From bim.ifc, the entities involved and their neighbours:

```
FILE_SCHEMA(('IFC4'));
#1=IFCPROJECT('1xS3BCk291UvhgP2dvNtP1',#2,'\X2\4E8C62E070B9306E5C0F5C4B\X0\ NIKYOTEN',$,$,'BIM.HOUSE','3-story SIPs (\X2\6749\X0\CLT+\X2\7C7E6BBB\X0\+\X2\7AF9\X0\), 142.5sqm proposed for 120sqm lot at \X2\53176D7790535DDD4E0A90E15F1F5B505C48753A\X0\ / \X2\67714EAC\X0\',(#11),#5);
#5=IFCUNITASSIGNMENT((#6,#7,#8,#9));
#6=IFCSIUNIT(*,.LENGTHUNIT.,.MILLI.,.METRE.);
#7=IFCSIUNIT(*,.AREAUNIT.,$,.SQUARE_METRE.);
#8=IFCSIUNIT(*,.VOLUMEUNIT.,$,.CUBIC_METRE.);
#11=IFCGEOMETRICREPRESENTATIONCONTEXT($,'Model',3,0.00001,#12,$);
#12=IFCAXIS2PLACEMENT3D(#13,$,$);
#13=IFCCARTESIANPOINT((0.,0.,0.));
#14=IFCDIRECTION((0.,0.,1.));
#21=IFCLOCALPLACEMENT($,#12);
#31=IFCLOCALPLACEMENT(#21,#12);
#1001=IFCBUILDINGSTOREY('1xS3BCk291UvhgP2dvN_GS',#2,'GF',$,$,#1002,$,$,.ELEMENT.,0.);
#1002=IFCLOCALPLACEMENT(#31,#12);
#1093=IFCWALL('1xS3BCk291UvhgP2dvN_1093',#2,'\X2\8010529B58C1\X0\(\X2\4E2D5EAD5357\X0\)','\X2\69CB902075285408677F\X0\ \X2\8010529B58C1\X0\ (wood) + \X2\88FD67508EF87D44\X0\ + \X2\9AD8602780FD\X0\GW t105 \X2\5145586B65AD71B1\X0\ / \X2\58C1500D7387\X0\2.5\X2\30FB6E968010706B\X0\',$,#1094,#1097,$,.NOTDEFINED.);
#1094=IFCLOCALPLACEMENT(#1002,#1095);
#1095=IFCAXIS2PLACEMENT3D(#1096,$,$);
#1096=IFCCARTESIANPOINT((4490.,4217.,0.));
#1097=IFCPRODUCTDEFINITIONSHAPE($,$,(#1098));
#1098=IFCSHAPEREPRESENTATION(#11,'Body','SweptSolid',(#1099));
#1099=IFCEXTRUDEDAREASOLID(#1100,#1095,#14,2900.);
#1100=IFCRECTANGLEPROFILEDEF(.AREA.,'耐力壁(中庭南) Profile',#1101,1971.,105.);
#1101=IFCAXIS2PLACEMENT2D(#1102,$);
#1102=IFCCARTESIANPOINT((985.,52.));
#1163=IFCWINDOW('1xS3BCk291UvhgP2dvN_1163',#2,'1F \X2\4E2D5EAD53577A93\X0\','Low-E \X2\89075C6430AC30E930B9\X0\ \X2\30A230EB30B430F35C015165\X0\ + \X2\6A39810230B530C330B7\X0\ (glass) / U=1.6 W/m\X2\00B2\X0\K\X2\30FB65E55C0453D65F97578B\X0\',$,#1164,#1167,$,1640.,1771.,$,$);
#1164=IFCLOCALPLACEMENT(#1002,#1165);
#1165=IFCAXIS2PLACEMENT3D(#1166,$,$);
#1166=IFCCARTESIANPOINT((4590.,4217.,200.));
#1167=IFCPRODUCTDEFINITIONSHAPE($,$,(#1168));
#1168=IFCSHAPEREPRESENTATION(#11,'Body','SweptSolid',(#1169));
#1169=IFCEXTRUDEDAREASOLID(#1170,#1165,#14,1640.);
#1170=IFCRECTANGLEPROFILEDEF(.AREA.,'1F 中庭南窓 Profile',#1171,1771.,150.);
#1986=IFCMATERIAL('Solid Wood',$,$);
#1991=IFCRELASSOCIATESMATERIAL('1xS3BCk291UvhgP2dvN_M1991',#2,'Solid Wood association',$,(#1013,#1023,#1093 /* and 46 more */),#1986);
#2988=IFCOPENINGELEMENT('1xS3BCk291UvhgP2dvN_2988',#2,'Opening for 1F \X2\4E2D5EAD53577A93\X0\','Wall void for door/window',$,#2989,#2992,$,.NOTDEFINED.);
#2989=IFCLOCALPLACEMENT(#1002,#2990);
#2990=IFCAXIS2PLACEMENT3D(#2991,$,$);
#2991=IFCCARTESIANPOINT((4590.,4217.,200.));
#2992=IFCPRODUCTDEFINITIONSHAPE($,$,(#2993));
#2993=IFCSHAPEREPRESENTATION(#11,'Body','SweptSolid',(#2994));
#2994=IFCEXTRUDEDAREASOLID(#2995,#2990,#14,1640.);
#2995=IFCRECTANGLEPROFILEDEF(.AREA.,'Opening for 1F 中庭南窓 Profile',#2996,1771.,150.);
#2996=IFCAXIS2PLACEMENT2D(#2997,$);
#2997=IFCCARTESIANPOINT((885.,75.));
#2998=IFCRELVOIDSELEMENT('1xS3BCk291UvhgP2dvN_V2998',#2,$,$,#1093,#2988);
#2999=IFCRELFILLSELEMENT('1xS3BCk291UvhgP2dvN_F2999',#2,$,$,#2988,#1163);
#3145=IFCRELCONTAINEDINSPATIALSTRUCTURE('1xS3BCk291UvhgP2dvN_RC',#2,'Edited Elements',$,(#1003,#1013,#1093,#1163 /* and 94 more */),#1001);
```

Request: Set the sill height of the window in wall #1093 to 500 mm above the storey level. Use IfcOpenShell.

```python
import numpy as np
import ifcopenshell
import ifcopenshell.api.geometry
import ifcopenshell.geom
import ifcopenshell.util.element
import ifcopenshell.util.placement
import ifcopenshell.util.shape
import ifcopenshell.util.unit

model = ifcopenshell.open("bim.ifc")
unit_scale = ifcopenshell.util.unit.calculate_unit_scale(model)

window = model.by_guid("1xS3BCk291UvhgP2dvN_1163")
opening = window.FillsVoids[0].RelatingOpeningElement
storey = ifcopenshell.util.element.get_container(window, ifc_class="IfcBuildingStorey")
level = ifcopenshell.util.placement.get_local_placement(storey.ObjectPlacement)[2, 3]

# The opening's origin need not be at the sill, so measure its lowest point.
shape = ifcopenshell.geom.create_shape(ifcopenshell.geom.settings(), opening)
bottom = ifcopenshell.util.shape.get_shape_bottom_elevation(shape, shape.geometry) / unit_scale
dz = level + 500.0 - bottom

shift = np.array([0.0, 0.0, dz])
# The window is not placed relative to its opening, so move both.
for product in (opening, window):
    matrix = ifcopenshell.util.placement.get_local_placement(product.ObjectPlacement)
    matrix[:3, 3] += shift
    ifcopenshell.api.geometry.edit_object_placement(model, product=product, matrix=matrix, is_si=False)

print(f"moved by {dz * unit_scale:+.3f} m")

model.write("bim_v2.ifc")
```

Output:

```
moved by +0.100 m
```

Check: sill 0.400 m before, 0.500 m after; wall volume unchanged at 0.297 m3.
